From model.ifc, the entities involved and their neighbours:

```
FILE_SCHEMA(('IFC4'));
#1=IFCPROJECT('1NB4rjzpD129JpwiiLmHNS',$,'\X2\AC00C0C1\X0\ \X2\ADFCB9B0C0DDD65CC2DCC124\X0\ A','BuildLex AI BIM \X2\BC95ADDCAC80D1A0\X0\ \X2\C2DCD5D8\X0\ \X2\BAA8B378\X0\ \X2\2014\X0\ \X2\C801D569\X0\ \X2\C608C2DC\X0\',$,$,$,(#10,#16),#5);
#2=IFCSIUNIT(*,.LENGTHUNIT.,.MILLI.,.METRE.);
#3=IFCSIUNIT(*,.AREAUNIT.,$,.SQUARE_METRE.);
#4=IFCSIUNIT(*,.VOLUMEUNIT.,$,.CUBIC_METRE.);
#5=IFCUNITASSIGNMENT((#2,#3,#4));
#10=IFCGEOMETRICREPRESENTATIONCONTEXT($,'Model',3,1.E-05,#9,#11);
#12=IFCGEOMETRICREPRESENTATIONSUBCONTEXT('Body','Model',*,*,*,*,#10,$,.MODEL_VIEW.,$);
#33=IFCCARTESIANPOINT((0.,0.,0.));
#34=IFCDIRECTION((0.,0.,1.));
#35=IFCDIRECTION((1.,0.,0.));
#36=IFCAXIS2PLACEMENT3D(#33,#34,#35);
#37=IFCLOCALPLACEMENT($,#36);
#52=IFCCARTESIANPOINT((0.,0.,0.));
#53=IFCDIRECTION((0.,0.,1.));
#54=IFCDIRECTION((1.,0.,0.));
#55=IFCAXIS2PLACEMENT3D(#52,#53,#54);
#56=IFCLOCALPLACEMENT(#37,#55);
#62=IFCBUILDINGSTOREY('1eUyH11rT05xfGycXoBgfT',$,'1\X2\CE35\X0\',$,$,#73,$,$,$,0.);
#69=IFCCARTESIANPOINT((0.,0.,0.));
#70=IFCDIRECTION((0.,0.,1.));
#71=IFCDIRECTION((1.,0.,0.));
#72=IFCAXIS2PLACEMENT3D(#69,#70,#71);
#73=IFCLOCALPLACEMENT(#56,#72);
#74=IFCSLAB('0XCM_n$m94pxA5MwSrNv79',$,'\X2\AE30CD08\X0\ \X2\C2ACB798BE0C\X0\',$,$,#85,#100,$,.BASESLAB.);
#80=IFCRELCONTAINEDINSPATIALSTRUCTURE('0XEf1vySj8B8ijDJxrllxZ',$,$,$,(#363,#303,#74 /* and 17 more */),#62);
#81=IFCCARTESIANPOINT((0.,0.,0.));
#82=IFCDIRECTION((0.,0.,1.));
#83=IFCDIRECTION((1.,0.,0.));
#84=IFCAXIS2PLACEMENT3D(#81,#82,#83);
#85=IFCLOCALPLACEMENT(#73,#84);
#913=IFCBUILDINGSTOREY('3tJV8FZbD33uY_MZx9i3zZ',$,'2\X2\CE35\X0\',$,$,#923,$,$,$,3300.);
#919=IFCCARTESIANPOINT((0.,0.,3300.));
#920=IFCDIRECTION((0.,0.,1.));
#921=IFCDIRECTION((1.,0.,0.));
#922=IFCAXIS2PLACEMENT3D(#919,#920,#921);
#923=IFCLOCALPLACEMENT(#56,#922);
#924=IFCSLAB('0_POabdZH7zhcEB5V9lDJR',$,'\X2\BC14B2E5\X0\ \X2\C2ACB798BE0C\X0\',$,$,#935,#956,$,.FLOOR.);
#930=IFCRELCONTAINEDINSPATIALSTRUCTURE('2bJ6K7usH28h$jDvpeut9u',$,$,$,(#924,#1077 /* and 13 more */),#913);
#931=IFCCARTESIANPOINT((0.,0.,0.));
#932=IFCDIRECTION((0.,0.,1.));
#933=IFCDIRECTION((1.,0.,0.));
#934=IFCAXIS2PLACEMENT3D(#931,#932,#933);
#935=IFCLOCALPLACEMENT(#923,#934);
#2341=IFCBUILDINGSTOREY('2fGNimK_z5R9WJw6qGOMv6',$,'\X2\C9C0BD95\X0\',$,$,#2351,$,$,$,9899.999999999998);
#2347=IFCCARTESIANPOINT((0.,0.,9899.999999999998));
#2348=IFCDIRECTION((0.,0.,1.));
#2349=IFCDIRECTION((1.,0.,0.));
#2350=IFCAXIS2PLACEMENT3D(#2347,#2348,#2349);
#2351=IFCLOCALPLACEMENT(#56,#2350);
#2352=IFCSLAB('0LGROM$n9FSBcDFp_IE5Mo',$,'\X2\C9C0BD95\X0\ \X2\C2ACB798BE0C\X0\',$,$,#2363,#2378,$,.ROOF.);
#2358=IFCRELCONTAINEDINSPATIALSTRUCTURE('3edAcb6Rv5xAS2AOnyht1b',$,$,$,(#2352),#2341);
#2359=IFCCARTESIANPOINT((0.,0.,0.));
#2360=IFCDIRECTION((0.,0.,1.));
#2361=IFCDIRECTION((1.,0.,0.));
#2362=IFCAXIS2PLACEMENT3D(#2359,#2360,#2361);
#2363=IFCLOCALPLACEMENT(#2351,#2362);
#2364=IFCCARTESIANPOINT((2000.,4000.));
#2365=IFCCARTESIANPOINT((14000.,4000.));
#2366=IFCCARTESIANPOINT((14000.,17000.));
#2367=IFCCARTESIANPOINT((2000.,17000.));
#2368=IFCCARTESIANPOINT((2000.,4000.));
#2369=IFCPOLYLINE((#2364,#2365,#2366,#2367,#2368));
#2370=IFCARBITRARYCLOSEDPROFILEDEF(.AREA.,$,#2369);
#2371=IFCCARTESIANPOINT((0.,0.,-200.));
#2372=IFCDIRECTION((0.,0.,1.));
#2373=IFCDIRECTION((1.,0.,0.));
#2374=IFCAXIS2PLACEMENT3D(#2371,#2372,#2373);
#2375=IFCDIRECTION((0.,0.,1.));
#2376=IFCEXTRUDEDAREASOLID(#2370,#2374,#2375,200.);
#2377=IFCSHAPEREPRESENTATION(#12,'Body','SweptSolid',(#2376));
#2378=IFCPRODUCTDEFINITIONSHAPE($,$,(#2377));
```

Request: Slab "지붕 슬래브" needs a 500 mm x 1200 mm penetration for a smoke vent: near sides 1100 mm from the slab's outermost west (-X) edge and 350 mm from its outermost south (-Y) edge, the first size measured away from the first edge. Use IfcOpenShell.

```python
import numpy as np
import ifcopenshell
import ifcopenshell.api.feature
import ifcopenshell.api.geometry
import ifcopenshell.api.root
import ifcopenshell.geom
import ifcopenshell.util.placement
import ifcopenshell.util.representation
import ifcopenshell.util.shape
import ifcopenshell.util.unit

model = ifcopenshell.open("model.ifc")
unit_scale = ifcopenshell.util.unit.calculate_unit_scale(model)
settings = ifcopenshell.geom.settings()


def volume(element):
    """Net volume in cubic metres, openings subtracted."""
    shape = ifcopenshell.geom.create_shape(settings, element)
    return ifcopenshell.util.shape.get_volume(shape.geometry)


slab = model.by_guid("0LGROM$n9FSBcDFp_IE5Mo")
before = volume(slab)

# Extent in the slab's own axes, in metres. The edges named are its -X and -Y sides.
slab_shape = ifcopenshell.geom.create_shape(settings, slab)
vertices = ifcopenshell.util.shape.get_vertices(slab_shape.geometry)
x_min, y_min, bottom = vertices.min(axis=0)
top = vertices[:, 2].max()

opening = ifcopenshell.api.root.create_entity(model, ifc_class="IfcOpeningElement", name="Smoke vent opening", predefined_type="OPENING")
context = ifcopenshell.util.representation.get_context(model, "Model", "Body", "MODEL_VIEW")
width, depth = 0.5, 1.2
outline = [(0.0, 0.0), (width, 0.0), (width, depth), (0.0, depth), (0.0, 0.0)]
# Overshoot both faces by 50 mm so the cut is clean.
shape = ifcopenshell.api.geometry.add_slab_representation(
    model, context=context, depth=top - bottom + 0.1, polyline=outline
)
ifcopenshell.api.geometry.assign_representation(model, product=opening, representation=shape)

matrix = ifcopenshell.util.placement.get_local_placement(slab.ObjectPlacement)
matrix[:, 3] = matrix @ np.append(np.array([x_min + 1.1, y_min + 0.35, bottom - 0.05]) / unit_scale, 1.0)
ifcopenshell.api.geometry.edit_object_placement(model, product=opening, matrix=matrix, is_si=False)
ifcopenshell.api.feature.add_feature(model, feature=opening, element=slab)

after = volume(slab)

print(f"slab volume {before:.3f} -> {after:.3f} m3")

model.write("model_v2.ifc")
```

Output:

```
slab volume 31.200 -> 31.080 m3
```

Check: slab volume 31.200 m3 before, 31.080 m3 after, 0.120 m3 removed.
